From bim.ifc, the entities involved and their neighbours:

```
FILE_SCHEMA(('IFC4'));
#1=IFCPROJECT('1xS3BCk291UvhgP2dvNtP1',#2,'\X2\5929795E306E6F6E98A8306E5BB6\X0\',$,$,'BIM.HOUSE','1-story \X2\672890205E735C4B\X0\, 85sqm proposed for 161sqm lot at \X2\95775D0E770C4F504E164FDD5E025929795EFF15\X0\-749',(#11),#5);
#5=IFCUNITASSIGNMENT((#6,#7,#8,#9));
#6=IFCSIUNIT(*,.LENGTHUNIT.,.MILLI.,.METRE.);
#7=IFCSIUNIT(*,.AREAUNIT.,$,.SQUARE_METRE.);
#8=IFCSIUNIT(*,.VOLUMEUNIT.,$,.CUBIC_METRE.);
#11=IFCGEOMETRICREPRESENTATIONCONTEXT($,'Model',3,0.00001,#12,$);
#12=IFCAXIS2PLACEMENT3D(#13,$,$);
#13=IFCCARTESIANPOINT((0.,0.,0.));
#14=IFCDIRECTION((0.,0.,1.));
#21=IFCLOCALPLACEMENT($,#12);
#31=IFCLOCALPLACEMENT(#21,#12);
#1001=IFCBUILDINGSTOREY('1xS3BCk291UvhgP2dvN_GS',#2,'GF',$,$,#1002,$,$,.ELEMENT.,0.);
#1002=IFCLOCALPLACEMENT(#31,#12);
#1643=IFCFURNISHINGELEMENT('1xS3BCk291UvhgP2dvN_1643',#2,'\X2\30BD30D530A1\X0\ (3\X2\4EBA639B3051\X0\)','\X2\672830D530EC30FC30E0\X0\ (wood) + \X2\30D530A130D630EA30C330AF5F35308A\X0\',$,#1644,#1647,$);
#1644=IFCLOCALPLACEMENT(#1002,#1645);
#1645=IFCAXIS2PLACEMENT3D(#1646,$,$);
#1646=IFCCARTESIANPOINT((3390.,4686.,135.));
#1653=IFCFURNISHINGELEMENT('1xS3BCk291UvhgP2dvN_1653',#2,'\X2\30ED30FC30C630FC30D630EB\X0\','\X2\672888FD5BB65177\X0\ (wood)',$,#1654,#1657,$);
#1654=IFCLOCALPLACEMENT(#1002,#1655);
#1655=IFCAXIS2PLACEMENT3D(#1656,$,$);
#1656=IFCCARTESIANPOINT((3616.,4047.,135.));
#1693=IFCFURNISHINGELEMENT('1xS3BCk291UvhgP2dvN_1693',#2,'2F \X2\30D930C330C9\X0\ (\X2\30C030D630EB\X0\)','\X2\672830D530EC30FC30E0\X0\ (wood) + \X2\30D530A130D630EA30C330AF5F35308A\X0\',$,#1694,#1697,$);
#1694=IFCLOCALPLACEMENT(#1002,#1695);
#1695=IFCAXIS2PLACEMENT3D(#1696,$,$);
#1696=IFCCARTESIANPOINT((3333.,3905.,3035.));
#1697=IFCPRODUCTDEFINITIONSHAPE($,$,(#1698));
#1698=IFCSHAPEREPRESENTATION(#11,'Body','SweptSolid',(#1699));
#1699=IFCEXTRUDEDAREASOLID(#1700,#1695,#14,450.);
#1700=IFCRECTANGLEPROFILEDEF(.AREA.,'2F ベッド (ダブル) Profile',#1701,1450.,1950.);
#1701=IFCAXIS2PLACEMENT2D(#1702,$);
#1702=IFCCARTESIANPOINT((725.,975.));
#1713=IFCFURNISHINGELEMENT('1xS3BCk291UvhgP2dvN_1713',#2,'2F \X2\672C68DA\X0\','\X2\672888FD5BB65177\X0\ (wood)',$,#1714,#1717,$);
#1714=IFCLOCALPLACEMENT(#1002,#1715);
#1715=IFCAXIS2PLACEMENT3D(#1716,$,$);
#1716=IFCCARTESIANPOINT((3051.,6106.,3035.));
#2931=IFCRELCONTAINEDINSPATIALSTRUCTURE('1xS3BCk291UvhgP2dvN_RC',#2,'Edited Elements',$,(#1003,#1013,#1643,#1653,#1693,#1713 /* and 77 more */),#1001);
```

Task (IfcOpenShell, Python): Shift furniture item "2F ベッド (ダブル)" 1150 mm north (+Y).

```python
import ifcopenshell
import ifcopenshell.api.geometry
import ifcopenshell.util.placement

model = ifcopenshell.open("bim.ifc")

item = model.by_guid("1xS3BCk291UvhgP2dvN_1693")
matrix = ifcopenshell.util.placement.get_local_placement(item.ObjectPlacement)
matrix[1, 3] += 1150.0
ifcopenshell.api.geometry.edit_object_placement(model, product=item, matrix=matrix, is_si=False)

print(ifcopenshell.util.placement.get_local_placement(item.ObjectPlacement).round(3) + 0.0)

model.write("bim_updated.ifc")
```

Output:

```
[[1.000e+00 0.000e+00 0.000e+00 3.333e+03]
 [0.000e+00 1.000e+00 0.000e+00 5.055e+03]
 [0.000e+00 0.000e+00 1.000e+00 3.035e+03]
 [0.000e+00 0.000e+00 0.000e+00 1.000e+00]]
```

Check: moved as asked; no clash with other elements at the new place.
